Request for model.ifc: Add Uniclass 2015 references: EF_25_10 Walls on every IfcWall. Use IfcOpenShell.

First a look at what the model holds.

```python
import ifcopenshell

model = ifcopenshell.open("model.ifc")
print(model.schema)
print("classifications:", [c.Name for c in model.by_type("IfcClassification")])
for ifc_class in ("IfcDoor", "IfcRoof", "IfcStair", "IfcWall", "IfcWindow"):
    print(ifc_class, len(model.by_type(ifc_class)))
```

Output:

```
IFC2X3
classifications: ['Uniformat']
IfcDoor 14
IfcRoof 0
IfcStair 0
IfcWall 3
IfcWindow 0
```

```python
import ifcopenshell
import ifcopenshell.api.classification

model = ifcopenshell.open("model.ifc")

# IFC2X3 requires Source and Edition and has no link from the project to the system.
system = model.create_entity("IfcClassification", Source="NBS", Edition="2015", Name="Uniclass 2015")

codes = {
    "IfcWall": ("EF_25_10", "Walls"),
}
for ifc_class, (code, name) in codes.items():
    products = model.by_type(ifc_class)
    ifcopenshell.api.classification.add_reference(
        model, products=products, classification=system, identification=code, name=name
    )
    print(code, len(products))

model.write("model_v2.ifc")
```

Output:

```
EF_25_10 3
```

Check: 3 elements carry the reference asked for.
